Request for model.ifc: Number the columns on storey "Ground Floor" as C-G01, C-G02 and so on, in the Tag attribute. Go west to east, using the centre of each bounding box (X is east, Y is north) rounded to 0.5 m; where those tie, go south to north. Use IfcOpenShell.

First a look at what the model holds.

```python
import ifcopenshell
import ifcopenshell.util.element
import ifcopenshell.util.placement

model = ifcopenshell.open("model.ifc")
print(model.schema)
storey = next(s for s in model.by_type("IfcBuildingStorey") if s.Name == "Ground Floor")
columns = [e for e in ifcopenshell.util.element.get_decomposition(storey) if e.is_a("IfcColumn")]
for e in sorted(columns, key=lambda e: e.id()):
    origin = ifcopenshell.util.placement.get_local_placement(e.ObjectPlacement)[:3, 3]
    print(e.id(), e.Tag, e.Name, origin.round(2) + 0.0, sep=" | ")
```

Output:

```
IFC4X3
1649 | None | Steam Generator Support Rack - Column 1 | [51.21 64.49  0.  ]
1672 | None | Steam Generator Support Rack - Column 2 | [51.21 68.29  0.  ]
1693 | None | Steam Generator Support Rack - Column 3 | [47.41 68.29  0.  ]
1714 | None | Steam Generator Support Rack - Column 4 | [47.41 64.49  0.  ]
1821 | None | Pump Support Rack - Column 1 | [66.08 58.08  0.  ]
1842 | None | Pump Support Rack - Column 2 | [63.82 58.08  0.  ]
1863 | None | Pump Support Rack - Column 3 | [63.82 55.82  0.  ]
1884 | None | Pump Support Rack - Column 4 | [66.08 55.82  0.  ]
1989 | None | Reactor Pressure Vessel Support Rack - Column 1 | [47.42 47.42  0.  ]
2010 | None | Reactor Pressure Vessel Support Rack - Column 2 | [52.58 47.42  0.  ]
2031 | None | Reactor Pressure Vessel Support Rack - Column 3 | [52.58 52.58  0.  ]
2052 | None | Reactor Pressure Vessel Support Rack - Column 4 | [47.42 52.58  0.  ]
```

```python
import ifcopenshell
import ifcopenshell.geom
import ifcopenshell.util.element
import ifcopenshell.util.shape

model = ifcopenshell.open("model.ifc")
settings = ifcopenshell.geom.settings()
settings.set("use-world-coords", True)


def centre(element):
    shape = ifcopenshell.geom.create_shape(settings, element)
    return ifcopenshell.util.shape.get_bbox_centroid(shape.geometry)


storey = next(s for s in model.by_type("IfcBuildingStorey") if s.Name == "Ground Floor")
columns = [e for e in ifcopenshell.util.element.get_decomposition(storey) if e.is_a("IfcColumn")]

# Insertion points can sit at a corner or the storey origin, so sort by the geometry (in metres).
centres = {e: centre(e) for e in columns}
columns.sort(key=lambda e: (round(centres[e][0] / 0.5), centres[e][1]))

for i, e in enumerate(columns, start=1):
    number = f"C-G{i:02d}"
    e.Tag = number
    print(e.id(), number)

model.write("model-out.ifc")
```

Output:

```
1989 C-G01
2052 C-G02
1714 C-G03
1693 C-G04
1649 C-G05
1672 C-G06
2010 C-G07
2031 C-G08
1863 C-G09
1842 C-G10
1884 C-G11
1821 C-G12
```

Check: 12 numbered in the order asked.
